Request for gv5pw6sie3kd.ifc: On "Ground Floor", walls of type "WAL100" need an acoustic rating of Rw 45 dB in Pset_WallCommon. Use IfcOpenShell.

First a look at what the model holds.

```python
import ifcopenshell
import ifcopenshell.util.element

model = ifcopenshell.open("gv5pw6sie3kd.ifc")
print(model.schema)
storey = next(s for s in model.by_type("IfcBuildingStorey") if s.Name == "Ground Floor")
walls = [e for e in ifcopenshell.util.element.get_decomposition(storey) if e.is_a("IfcWall")]
seen = {}
for e in walls:
    element_type = ifcopenshell.util.element.get_type(e)
    key = (element_type.Name if element_type != e and element_type else None, ifcopenshell.util.element.get_pset(e, "Pset_WallCommon", "AcousticRating"))
    seen[key] = seen.get(key, 0) + 1
for (name, value), count in sorted(seen.items(), key=str):
    print(count, "x", name, "|", value)
```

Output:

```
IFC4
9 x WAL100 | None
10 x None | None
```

```python
import ifcopenshell
import ifcopenshell.api.pset
import ifcopenshell.util.element

model = ifcopenshell.open("gv5pw6sie3kd.ifc")

storey = next(s for s in model.by_type("IfcBuildingStorey") if s.Name == "Ground Floor")
walls = [e for e in ifcopenshell.util.element.get_decomposition(storey) if e.is_a("IfcWall")]

count = 0
for e in walls:
    element_type = ifcopenshell.util.element.get_type(e)
    if element_type in (None, e) or element_type.Name != "WAL100":
        continue
    # add_pset returns the element's existing set when there is one.
    pset = ifcopenshell.api.pset.add_pset(model, product=e, name="Pset_WallCommon")
    ifcopenshell.api.pset.edit_pset(model, pset=pset, properties={"AcousticRating": "Rw 45 dB"})
    count += 1

print(count, "walls updated")

model.write("gv5pw6sie3kd_v2.ifc")
```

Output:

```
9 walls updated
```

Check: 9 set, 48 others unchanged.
